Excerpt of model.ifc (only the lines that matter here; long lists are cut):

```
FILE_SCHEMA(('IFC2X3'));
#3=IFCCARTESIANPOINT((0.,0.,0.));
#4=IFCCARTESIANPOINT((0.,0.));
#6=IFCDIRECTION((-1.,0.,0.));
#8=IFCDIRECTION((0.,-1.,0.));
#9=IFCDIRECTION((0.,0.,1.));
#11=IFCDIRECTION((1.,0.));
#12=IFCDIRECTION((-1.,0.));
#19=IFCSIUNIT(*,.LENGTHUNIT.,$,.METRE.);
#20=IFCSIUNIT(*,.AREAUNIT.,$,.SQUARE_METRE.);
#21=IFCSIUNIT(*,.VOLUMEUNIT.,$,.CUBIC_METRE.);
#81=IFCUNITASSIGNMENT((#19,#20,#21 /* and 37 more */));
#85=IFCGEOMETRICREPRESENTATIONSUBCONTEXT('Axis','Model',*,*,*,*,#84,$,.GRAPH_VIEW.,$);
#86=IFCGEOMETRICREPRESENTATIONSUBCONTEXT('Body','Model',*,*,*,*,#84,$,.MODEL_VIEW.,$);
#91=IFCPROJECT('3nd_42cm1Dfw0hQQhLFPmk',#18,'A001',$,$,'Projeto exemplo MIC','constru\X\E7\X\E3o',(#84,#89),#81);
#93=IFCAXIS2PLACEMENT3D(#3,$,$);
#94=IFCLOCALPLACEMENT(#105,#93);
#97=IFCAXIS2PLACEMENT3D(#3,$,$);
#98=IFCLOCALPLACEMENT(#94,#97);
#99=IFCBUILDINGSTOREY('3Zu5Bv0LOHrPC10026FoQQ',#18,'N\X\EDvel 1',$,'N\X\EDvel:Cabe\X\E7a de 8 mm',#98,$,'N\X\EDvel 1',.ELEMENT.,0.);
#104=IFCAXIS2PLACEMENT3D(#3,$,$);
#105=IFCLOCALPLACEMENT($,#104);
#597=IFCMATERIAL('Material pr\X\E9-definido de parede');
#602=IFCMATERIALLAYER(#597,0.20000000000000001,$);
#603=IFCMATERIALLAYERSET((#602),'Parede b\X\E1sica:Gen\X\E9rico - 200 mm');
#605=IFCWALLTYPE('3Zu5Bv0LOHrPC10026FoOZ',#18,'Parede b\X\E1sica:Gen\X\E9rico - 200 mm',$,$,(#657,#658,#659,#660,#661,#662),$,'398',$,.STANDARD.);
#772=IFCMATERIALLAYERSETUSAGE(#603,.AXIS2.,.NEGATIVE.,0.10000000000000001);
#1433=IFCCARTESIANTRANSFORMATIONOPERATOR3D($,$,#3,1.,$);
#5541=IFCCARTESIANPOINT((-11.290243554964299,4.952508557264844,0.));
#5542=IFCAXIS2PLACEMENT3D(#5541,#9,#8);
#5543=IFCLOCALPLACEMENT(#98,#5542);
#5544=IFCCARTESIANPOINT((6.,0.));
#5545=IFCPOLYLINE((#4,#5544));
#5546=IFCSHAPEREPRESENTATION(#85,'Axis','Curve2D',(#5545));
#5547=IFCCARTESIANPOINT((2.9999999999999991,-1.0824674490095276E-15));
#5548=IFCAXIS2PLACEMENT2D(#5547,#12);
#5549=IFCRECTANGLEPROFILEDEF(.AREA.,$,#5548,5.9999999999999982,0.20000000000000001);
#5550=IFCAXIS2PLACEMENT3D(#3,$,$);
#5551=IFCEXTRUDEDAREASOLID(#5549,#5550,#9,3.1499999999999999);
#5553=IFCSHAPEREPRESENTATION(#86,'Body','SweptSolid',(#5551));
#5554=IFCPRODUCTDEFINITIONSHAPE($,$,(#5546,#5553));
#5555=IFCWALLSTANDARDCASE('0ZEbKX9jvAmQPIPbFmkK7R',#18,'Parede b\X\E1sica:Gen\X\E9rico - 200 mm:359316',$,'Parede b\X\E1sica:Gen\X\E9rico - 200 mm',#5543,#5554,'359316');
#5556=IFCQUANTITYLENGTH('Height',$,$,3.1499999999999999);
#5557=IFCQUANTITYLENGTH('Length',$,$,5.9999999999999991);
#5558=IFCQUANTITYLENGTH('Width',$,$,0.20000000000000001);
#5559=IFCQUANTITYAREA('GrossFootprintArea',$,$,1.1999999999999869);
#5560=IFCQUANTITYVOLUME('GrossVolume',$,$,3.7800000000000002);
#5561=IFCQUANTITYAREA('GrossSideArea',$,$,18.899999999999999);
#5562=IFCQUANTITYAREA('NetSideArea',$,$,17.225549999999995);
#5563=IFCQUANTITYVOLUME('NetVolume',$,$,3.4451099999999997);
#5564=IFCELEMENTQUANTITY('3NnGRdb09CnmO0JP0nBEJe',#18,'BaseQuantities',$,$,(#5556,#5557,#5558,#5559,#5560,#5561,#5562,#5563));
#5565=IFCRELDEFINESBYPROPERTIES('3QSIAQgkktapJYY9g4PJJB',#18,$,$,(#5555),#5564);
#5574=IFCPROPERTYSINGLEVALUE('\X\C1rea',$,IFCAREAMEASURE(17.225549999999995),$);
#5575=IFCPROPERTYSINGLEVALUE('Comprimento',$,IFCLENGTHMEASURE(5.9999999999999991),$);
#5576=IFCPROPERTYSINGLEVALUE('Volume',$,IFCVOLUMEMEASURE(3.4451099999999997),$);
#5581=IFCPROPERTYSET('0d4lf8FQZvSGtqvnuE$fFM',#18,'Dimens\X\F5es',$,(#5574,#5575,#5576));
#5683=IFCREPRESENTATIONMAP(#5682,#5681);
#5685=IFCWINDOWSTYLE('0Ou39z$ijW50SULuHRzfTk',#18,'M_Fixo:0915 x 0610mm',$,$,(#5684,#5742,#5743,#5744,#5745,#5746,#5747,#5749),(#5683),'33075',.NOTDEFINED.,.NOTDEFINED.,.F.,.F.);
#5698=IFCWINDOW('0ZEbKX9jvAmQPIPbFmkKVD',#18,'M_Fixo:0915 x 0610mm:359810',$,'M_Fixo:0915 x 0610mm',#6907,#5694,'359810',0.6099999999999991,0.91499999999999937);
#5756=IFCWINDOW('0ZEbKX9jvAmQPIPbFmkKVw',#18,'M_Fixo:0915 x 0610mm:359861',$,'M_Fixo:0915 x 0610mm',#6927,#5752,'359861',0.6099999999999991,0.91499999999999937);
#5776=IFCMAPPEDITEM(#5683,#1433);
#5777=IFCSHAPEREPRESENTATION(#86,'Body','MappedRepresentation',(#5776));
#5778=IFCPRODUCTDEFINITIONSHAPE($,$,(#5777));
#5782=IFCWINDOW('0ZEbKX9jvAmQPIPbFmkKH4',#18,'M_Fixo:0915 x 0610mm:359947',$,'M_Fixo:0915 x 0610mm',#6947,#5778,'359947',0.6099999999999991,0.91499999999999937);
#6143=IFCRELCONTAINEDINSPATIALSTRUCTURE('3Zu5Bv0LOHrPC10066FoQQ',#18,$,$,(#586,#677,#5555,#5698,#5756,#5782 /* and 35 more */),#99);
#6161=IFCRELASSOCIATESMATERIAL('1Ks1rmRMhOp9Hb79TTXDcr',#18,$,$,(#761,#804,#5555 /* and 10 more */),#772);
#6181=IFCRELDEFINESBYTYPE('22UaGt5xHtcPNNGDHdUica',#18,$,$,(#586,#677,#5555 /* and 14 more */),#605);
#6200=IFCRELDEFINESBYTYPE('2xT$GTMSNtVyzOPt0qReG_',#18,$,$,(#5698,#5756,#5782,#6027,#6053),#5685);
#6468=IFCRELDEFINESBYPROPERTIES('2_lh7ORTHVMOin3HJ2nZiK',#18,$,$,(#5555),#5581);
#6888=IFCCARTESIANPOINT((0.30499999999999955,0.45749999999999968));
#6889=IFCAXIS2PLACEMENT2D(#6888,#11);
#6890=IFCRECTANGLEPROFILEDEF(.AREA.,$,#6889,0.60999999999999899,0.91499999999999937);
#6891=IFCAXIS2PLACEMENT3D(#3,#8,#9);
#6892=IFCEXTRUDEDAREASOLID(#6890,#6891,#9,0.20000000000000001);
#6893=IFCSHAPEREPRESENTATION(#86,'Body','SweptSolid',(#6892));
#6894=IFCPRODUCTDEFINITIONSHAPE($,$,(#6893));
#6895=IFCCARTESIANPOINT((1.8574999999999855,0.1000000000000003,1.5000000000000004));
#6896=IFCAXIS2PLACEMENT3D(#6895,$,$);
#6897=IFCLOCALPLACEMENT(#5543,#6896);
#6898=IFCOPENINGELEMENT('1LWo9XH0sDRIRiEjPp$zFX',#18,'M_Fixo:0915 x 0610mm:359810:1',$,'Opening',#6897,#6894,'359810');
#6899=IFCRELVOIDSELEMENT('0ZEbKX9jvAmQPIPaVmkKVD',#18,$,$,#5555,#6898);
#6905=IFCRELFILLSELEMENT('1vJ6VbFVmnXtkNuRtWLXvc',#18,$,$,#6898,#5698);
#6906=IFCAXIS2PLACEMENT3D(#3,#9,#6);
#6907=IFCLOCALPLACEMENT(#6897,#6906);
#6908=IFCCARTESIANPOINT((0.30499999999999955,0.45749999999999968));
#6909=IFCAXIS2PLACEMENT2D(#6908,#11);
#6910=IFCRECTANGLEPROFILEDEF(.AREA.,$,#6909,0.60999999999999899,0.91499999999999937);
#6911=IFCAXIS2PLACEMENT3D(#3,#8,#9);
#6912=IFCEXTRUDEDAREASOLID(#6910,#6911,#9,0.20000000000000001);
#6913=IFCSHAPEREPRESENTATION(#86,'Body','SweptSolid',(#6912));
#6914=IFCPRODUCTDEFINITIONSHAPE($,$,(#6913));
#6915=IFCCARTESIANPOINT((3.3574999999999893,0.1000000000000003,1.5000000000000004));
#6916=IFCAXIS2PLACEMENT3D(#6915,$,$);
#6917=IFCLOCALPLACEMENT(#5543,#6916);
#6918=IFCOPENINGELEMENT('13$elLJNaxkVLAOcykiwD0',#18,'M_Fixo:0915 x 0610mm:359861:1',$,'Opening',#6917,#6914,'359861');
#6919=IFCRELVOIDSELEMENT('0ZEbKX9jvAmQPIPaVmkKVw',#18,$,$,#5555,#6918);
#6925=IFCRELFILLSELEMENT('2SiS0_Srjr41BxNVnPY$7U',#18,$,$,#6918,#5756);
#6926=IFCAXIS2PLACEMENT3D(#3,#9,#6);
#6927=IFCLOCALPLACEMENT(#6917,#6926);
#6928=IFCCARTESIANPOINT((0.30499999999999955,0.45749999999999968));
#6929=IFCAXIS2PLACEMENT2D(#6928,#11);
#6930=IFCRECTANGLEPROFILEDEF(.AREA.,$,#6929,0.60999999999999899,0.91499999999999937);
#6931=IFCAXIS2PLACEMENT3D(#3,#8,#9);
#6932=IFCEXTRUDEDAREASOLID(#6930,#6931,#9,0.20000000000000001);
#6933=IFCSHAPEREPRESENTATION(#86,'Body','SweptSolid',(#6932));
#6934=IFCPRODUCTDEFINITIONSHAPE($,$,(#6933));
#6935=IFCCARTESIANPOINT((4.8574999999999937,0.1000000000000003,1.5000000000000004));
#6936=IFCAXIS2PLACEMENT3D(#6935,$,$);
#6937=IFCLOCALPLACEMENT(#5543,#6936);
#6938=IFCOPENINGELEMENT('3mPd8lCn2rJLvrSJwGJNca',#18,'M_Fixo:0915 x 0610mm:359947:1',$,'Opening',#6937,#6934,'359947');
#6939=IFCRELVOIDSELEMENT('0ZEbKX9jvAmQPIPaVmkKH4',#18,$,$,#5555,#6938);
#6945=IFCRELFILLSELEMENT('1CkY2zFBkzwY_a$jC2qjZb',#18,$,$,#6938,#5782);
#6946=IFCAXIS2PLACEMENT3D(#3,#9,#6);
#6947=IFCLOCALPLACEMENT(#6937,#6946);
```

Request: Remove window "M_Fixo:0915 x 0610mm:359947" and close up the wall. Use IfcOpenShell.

```python
import ifcopenshell
import ifcopenshell.api.feature
import ifcopenshell.api.pset
import ifcopenshell.api.root
import ifcopenshell.geom
import ifcopenshell.util.element
import ifcopenshell.util.shape
import ifcopenshell.util.unit

model = ifcopenshell.open("model.ifc")
area_scale = ifcopenshell.util.unit.calculate_unit_scale(model, "AREAUNIT")
volume_scale = ifcopenshell.util.unit.calculate_unit_scale(model, "VOLUMEUNIT")
settings = ifcopenshell.geom.settings()


def volume(element):
    """Net volume in cubic metres, openings subtracted."""
    shape = ifcopenshell.geom.create_shape(settings, element)
    return ifcopenshell.util.shape.get_volume(shape.geometry)


window = model.by_id(5782)
opening = window.FillsVoids[0].RelatingOpeningElement
wall = opening.VoidsElements[0].RelatingBuildingElement
before = volume(wall)

ifcopenshell.api.root.remove_product(model, product=window)
ifcopenshell.api.feature.remove_feature(model, feature=opening)

after = volume(wall)
thickness = 0.2  # wall thickness in metres

# Update the wall's stored quantities.
qto = model.by_id(ifcopenshell.util.element.get_pset(wall, "BaseQuantities", should_inherit=False)["id"])
ifcopenshell.api.pset.edit_qto(model, qto=qto, properties={
    "NetSideArea": after / thickness / area_scale,
    "NetVolume": after / volume_scale,
})
pset = model.by_id(ifcopenshell.util.element.get_pset(wall, "Dimensões", should_inherit=False)["id"])
ifcopenshell.api.pset.edit_pset(model, pset=pset, properties={
    "Área": model.create_entity("IfcAreaMeasure", after / thickness / area_scale),
    "Volume": model.create_entity("IfcVolumeMeasure", after / volume_scale),
})

print(f"wall volume {before:.3f} -> {after:.3f} m3")

model.write("model_updated.ifc")
```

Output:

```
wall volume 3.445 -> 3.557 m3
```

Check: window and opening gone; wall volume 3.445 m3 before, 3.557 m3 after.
